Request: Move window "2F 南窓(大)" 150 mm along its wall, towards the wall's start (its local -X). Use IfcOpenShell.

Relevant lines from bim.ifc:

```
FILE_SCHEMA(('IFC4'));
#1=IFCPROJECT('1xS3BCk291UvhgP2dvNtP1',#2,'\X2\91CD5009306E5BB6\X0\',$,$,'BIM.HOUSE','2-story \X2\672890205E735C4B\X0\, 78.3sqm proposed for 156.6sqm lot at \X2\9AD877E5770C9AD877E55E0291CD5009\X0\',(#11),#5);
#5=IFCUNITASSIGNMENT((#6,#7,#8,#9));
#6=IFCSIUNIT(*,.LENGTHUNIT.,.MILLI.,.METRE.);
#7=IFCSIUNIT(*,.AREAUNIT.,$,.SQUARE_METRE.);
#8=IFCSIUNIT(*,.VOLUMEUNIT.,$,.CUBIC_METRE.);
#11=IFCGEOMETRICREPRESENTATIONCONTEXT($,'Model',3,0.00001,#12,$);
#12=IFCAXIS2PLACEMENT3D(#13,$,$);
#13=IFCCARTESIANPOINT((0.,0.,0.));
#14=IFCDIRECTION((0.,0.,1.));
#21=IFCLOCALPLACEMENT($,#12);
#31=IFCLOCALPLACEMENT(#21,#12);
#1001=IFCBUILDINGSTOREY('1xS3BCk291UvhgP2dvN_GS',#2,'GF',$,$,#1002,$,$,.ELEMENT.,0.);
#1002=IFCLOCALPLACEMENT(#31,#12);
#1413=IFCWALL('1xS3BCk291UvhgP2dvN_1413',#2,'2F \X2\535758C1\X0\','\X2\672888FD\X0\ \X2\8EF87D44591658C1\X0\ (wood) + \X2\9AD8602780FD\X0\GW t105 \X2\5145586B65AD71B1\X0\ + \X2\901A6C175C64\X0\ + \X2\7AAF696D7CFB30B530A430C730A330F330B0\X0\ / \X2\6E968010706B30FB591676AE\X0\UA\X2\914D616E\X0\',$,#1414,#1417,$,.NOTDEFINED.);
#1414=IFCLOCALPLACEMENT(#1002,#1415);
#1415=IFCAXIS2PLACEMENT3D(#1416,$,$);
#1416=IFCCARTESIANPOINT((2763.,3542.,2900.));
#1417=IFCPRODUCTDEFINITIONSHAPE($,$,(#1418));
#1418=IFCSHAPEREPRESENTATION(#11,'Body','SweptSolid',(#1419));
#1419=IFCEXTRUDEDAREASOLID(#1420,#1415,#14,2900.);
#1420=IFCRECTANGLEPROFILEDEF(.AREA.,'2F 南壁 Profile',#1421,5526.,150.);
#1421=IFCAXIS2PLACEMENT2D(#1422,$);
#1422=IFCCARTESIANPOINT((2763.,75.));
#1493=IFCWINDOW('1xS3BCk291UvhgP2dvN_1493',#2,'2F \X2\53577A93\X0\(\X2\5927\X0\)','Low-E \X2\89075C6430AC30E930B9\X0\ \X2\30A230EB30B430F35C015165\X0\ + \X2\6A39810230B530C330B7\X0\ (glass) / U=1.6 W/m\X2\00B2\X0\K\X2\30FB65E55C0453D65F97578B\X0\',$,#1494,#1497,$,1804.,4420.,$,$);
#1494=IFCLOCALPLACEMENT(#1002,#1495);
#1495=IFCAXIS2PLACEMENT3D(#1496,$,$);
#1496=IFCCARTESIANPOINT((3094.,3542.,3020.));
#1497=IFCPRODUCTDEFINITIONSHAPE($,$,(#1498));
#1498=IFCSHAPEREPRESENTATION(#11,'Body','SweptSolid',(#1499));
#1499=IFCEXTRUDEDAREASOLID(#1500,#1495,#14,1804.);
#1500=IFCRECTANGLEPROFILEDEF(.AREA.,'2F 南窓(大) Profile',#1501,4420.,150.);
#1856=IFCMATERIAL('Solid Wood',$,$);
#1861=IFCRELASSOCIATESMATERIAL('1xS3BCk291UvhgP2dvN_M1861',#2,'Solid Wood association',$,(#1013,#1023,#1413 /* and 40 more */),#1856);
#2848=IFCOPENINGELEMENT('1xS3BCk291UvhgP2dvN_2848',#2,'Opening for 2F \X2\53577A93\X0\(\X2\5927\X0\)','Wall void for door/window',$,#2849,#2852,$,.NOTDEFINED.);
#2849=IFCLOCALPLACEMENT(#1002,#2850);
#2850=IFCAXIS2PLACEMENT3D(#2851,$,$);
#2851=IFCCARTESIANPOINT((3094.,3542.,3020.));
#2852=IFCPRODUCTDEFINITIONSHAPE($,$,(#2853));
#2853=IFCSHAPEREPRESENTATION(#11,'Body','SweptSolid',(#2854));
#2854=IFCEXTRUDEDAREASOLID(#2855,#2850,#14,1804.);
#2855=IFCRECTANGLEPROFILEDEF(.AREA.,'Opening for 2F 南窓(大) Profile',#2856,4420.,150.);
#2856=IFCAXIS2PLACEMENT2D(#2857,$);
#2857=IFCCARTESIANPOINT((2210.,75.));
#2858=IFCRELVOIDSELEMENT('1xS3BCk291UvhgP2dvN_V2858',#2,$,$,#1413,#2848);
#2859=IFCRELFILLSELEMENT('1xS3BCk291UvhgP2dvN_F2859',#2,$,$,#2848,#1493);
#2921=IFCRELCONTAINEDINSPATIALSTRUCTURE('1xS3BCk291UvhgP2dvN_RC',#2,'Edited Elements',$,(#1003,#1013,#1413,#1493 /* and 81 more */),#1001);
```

```python
import ifcopenshell
import ifcopenshell.api.geometry
import ifcopenshell.util.placement

model = ifcopenshell.open("bim.ifc")

window = model.by_id(1493)
opening = window.FillsVoids[0].RelatingOpeningElement
wall = opening.VoidsElements[0].RelatingBuildingElement

wall_matrix = ifcopenshell.util.placement.get_local_placement(wall.ObjectPlacement)
shift = wall_matrix[:3, 0] * -150.0
before = ifcopenshell.util.placement.get_local_placement(window.ObjectPlacement)[:3, 3].copy()

# The window is not placed relative to its opening, so move both.
for product in (opening, window):
    matrix = ifcopenshell.util.placement.get_local_placement(product.ObjectPlacement)
    matrix[:3, 3] += shift
    ifcopenshell.api.geometry.edit_object_placement(model, product=product, matrix=matrix, is_si=False)

after = ifcopenshell.util.placement.get_local_placement(window.ObjectPlacement)[:3, 3]
print("window moved by", (after - before).round(3) + 0.0)

model.write("bim_updated.ifc")
```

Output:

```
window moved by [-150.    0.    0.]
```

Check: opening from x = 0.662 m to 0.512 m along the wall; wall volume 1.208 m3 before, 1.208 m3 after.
